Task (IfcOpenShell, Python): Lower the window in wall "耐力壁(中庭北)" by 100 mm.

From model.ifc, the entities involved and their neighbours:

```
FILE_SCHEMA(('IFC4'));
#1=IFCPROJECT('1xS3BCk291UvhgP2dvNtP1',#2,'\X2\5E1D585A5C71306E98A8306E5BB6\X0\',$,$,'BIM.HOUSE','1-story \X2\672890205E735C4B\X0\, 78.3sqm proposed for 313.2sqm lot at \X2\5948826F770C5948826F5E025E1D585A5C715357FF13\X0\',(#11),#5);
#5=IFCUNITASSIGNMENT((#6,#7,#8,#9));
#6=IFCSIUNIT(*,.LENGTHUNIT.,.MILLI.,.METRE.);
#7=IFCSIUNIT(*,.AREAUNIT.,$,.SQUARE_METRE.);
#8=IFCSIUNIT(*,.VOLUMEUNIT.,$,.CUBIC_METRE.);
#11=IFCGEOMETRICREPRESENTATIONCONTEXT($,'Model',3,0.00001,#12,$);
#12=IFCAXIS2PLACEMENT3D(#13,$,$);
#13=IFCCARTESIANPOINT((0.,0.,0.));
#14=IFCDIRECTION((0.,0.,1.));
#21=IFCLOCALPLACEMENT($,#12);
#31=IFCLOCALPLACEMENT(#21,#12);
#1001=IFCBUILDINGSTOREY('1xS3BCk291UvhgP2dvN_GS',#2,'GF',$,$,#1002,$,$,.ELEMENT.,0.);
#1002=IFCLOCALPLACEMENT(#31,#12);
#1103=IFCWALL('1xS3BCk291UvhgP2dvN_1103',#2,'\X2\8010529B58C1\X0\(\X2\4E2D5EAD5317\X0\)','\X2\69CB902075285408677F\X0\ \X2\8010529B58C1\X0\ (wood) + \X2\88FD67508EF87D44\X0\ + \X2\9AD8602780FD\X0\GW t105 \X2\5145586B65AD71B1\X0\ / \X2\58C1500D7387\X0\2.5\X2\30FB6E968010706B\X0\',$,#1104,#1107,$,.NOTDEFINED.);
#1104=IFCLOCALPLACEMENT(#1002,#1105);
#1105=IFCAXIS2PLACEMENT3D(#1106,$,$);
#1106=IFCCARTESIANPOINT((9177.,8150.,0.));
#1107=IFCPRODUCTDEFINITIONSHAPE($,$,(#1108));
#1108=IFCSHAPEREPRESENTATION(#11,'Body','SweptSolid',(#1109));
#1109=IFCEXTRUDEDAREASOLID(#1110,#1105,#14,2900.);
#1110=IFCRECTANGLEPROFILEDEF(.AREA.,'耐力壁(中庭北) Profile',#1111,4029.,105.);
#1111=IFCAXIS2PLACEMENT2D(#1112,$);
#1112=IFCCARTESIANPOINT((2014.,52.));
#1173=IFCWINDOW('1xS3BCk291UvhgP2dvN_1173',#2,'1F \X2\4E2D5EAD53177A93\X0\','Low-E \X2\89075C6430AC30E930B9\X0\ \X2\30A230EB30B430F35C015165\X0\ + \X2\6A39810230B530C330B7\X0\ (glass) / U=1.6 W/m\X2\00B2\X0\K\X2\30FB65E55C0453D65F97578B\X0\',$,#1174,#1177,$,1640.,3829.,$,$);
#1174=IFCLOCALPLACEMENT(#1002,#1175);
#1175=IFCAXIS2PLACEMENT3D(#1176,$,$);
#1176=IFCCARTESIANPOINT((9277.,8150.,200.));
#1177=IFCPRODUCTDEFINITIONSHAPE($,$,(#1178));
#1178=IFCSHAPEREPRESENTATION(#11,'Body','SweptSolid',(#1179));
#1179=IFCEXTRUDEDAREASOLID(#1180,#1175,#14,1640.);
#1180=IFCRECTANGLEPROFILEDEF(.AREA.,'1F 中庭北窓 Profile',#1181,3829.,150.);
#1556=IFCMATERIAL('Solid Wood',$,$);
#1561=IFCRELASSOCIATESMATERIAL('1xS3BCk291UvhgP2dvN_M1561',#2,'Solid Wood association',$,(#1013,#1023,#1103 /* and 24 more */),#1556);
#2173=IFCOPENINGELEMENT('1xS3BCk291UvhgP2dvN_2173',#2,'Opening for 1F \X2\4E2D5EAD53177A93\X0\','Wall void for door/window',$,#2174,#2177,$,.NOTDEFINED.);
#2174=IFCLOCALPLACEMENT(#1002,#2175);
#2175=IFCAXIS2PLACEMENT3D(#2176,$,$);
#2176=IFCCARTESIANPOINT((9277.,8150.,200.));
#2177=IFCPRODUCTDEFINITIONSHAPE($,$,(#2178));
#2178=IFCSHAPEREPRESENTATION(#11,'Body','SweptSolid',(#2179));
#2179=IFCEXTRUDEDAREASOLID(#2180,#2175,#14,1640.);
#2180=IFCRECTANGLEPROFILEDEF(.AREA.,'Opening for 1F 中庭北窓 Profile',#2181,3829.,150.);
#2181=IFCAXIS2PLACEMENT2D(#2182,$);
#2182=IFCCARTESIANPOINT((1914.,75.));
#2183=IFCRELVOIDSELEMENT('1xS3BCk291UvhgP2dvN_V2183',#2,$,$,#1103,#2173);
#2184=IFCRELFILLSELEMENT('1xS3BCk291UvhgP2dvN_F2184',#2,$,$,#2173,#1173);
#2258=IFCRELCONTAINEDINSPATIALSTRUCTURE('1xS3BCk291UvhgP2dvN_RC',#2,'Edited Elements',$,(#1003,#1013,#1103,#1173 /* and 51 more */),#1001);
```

```python
import numpy as np
import ifcopenshell
import ifcopenshell.api.geometry
import ifcopenshell.util.placement
import ifcopenshell.util.unit

model = ifcopenshell.open("model.ifc")
unit_scale = ifcopenshell.util.unit.calculate_unit_scale(model)

window = model.by_guid("1xS3BCk291UvhgP2dvN_1173")
opening = window.FillsVoids[0].RelatingOpeningElement
dz = -100.0

shift = np.array([0.0, 0.0, dz])
# The window is not placed relative to its opening, so move both.
for product in (opening, window):
    matrix = ifcopenshell.util.placement.get_local_placement(product.ObjectPlacement)
    matrix[:3, 3] += shift
    ifcopenshell.api.geometry.edit_object_placement(model, product=product, matrix=matrix, is_si=False)

print(f"moved by {dz * unit_scale:+.3f} m")

model.write("model_updated.ifc")
```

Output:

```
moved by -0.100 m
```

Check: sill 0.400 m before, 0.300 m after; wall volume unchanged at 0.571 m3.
